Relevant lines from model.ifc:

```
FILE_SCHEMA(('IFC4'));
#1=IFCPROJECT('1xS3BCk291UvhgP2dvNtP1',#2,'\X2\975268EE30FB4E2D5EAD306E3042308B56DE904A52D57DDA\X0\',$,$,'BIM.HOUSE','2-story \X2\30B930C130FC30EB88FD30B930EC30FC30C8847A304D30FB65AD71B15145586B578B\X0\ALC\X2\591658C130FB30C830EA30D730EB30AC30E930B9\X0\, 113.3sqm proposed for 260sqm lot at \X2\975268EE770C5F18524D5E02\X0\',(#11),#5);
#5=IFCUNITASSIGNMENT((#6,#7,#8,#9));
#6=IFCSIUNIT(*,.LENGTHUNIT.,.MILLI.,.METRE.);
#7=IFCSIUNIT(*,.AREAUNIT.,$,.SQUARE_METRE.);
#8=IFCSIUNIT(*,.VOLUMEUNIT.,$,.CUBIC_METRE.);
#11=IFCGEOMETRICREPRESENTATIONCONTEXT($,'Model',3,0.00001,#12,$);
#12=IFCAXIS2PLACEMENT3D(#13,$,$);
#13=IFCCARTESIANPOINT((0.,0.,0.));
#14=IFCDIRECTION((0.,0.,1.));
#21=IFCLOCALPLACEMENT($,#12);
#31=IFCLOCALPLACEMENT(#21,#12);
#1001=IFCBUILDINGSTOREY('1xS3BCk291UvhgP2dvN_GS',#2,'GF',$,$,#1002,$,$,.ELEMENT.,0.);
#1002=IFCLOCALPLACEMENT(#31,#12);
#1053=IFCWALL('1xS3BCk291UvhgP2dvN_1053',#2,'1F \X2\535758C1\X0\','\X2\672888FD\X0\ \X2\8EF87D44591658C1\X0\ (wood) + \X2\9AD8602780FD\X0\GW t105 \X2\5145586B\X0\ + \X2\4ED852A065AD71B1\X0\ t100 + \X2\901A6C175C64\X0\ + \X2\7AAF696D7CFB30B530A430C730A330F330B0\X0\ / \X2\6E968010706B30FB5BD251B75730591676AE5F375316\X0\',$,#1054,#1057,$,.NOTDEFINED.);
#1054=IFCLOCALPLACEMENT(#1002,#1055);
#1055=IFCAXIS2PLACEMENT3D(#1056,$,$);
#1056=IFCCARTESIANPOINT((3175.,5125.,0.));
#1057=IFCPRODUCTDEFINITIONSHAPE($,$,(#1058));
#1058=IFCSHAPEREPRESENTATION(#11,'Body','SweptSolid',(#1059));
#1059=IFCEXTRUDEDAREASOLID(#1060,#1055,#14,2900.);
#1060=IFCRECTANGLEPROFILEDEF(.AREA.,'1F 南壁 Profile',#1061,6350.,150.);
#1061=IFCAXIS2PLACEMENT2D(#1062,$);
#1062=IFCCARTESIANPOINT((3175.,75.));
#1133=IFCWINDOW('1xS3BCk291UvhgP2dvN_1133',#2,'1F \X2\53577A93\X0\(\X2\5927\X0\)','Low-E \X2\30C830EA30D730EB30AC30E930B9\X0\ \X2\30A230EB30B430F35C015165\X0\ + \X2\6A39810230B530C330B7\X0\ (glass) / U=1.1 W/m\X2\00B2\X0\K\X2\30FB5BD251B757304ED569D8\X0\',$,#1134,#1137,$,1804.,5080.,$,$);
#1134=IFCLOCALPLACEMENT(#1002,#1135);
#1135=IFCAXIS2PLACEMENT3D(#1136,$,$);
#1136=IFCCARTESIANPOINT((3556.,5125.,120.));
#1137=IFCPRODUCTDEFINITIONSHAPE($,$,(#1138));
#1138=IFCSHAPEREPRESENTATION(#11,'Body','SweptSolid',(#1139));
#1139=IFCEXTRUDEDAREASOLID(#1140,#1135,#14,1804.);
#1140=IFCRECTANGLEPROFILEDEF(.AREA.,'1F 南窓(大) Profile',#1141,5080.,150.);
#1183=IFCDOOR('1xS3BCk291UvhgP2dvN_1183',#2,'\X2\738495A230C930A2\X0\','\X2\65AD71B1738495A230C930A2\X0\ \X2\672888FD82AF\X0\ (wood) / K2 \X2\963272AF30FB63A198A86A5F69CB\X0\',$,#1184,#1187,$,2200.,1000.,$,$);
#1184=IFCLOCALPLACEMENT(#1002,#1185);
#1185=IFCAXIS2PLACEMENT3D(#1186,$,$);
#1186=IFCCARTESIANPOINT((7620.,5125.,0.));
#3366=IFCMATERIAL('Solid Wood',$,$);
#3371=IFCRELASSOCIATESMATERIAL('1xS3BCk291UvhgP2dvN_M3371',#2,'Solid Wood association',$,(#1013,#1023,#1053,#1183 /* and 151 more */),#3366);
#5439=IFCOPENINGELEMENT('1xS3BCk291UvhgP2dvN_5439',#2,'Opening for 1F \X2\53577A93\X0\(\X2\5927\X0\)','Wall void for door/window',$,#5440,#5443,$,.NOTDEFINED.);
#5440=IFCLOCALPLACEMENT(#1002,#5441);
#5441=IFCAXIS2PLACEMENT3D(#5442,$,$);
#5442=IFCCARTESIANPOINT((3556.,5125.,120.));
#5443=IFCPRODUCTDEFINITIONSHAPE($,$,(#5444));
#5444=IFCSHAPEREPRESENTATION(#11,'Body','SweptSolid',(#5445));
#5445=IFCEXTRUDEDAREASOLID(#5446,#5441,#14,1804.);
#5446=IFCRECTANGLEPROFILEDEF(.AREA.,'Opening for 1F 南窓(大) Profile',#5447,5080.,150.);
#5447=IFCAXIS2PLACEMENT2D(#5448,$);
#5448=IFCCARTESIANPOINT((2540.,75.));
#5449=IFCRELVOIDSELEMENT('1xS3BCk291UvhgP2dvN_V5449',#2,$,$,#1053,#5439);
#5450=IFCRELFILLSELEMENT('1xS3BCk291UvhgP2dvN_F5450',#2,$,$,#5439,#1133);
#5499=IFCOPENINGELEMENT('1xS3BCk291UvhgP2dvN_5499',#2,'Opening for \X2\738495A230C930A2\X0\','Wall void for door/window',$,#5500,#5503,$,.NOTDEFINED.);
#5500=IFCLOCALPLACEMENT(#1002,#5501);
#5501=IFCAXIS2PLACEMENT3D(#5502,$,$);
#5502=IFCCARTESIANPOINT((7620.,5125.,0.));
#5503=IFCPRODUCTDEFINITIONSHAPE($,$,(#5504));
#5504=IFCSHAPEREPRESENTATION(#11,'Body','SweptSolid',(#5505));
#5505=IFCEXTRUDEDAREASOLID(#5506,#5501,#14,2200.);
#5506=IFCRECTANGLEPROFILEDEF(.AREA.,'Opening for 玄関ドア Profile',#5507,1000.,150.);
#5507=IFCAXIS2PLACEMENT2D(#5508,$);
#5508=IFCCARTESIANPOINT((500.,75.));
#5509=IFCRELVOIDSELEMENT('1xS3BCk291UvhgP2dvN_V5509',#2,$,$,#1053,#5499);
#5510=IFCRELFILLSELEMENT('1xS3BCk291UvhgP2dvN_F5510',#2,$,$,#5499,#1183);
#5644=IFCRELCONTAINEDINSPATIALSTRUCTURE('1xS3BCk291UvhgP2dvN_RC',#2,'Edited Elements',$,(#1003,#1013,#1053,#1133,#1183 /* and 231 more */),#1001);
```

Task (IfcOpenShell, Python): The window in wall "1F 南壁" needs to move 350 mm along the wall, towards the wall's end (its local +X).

```python
import ifcopenshell
import ifcopenshell.api.geometry
import ifcopenshell.util.placement
import ifcopenshell.util.unit

model = ifcopenshell.open("model.ifc")
unit_scale = ifcopenshell.util.unit.calculate_unit_scale(model)

window = model.by_guid("1xS3BCk291UvhgP2dvN_1133")
opening = window.FillsVoids[0].RelatingOpeningElement
wall = opening.VoidsElements[0].RelatingBuildingElement

wall_matrix = ifcopenshell.util.placement.get_local_placement(wall.ObjectPlacement)
shift = wall_matrix[:3, 0] * 0.35 / unit_scale
before = ifcopenshell.util.placement.get_local_placement(window.ObjectPlacement)[:3, 3].copy()

# The window is not placed relative to its opening, so move both.
for product in (opening, window):
    matrix = ifcopenshell.util.placement.get_local_placement(product.ObjectPlacement)
    matrix[:3, 3] += shift
    ifcopenshell.api.geometry.edit_object_placement(model, product=product, matrix=matrix, is_si=False)

after = ifcopenshell.util.placement.get_local_placement(window.ObjectPlacement)[:3, 3]
print("window moved by", (after - before).round(3) + 0.0)

model.write("model_v2.ifc")
```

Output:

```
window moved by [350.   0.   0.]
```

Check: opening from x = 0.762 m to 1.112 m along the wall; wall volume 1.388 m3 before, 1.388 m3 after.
